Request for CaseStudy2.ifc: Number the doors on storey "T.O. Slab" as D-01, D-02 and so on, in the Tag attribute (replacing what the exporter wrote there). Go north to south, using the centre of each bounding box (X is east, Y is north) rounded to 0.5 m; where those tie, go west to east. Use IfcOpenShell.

First a look at what the model holds.

```python
import ifcopenshell
import ifcopenshell.util.element
import ifcopenshell.util.placement

model = ifcopenshell.open("CaseStudy2.ifc")
print(model.schema)
storey = next(s for s in model.by_type("IfcBuildingStorey") if s.Name == "T.O. Slab")
doors = [e for e in ifcopenshell.util.element.get_decomposition(storey) if e.is_a("IfcDoor")]
for e in sorted(doors, key=lambda e: e.id()):
    origin = ifcopenshell.util.placement.get_local_placement(e.ObjectPlacement)[:3, 3]
    print(e.id(), e.Tag, e.Name, origin.round(2) + 0.0, sep=" | ")
```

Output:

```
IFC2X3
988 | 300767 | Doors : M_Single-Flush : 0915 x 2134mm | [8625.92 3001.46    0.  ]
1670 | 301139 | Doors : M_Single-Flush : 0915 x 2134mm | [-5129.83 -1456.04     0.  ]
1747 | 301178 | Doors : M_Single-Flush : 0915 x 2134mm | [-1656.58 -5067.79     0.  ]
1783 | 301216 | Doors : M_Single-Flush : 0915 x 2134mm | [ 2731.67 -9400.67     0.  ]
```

```python
import ifcopenshell
import ifcopenshell.geom
import ifcopenshell.util.element
import ifcopenshell.util.shape

model = ifcopenshell.open("CaseStudy2.ifc")
settings = ifcopenshell.geom.settings()
settings.set("use-world-coords", True)


def centre(element):
    shape = ifcopenshell.geom.create_shape(settings, element)
    return ifcopenshell.util.shape.get_bbox_centroid(shape.geometry)


storey = next(s for s in model.by_type("IfcBuildingStorey") if s.Name == "T.O. Slab")
doors = [e for e in ifcopenshell.util.element.get_decomposition(storey) if e.is_a("IfcDoor")]

# Insertion points can sit at a corner or the storey origin, so sort by the geometry (in metres).
centres = {e: centre(e) for e in doors}
doors.sort(key=lambda e: (-round(centres[e][1] / 0.5), centres[e][0]))

for i, e in enumerate(doors, start=1):
    number = f"D-{i:02d}"
    e.Tag = number
    print(e.id(), number)

model.write("CaseStudy2_updated.ifc")
```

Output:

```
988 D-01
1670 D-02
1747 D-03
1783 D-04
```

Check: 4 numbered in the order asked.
